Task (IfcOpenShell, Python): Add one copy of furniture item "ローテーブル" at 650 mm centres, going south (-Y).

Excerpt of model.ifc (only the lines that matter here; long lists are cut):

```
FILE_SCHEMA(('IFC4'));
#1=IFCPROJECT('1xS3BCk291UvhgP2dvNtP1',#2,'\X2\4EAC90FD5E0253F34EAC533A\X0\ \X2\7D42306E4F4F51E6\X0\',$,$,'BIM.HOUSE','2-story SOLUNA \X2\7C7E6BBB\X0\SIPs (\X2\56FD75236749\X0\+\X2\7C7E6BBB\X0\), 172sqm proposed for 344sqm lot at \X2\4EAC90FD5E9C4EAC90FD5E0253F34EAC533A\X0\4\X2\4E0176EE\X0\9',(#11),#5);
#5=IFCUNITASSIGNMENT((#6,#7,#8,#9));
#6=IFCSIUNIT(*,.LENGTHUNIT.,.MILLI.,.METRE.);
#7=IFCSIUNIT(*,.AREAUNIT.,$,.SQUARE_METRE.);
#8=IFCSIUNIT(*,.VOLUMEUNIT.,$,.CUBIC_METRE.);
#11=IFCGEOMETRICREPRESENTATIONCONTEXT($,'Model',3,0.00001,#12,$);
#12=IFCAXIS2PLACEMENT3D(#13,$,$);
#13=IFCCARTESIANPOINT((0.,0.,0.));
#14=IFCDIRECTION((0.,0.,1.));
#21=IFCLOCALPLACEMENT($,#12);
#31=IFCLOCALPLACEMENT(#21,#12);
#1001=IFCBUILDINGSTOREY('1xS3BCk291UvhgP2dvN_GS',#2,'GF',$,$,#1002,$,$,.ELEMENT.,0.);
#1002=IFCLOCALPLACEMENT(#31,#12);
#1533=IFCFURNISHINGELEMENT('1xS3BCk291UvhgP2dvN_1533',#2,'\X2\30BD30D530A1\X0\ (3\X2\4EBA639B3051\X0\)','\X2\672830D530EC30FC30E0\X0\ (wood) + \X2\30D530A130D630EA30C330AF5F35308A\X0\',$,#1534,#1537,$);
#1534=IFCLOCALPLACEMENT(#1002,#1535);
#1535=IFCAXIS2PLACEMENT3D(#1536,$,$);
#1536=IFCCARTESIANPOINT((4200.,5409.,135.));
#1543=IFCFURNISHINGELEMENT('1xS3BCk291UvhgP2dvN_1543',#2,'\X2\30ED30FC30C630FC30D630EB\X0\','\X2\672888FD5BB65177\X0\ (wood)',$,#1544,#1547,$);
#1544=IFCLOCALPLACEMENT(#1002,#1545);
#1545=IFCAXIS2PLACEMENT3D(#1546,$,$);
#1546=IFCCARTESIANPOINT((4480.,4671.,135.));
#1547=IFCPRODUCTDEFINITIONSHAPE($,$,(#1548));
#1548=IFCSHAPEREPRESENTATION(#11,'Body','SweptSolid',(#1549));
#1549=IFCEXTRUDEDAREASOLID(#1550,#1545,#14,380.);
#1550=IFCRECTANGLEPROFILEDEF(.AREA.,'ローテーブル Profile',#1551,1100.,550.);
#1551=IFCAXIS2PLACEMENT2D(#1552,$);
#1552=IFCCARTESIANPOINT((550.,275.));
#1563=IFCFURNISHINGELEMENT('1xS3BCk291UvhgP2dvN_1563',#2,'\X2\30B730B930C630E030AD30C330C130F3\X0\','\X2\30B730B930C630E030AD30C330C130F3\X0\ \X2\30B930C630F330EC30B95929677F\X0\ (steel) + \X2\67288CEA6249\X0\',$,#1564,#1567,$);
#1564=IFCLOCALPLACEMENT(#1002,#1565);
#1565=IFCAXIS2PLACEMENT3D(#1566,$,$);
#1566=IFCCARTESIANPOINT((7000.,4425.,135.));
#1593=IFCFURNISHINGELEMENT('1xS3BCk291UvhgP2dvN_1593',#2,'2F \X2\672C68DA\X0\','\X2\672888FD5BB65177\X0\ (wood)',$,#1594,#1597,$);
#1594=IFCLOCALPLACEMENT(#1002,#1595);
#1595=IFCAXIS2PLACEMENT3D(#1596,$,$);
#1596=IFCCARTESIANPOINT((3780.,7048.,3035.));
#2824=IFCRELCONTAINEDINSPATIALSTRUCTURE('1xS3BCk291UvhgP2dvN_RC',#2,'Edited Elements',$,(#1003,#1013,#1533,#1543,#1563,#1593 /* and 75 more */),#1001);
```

```python
import numpy as np
import ifcopenshell
import ifcopenshell.api.geometry
import ifcopenshell.api.root
import ifcopenshell.util.element
import ifcopenshell.util.placement
import ifcopenshell.util.unit

model = ifcopenshell.open("model.ifc")
unit_scale = ifcopenshell.util.unit.calculate_unit_scale(model)


def reuse_history(source, copy):
    """copy_class also copies each property set's owner history, people and application; keep the originals."""
    for rel in copy.IsDefinedBy:
        if rel.is_a("IfcRelDefinesByProperties") and (history := rel.RelatingPropertyDefinition.OwnerHistory):
            rel.RelatingPropertyDefinition.OwnerHistory = source.OwnerHistory
            ifcopenshell.util.element.remove_deep2(model, history)


source = model.by_id(1543)
base = ifcopenshell.util.placement.get_local_placement(source.ObjectPlacement)
step = np.array([0.0, -1.0, 0.0]) * 0.65 / unit_scale

for i in range(1, 2):
    copy = ifcopenshell.api.root.copy_class(model, product=source)
    copy.Representation = ifcopenshell.util.element.copy_deep(
        model, source.Representation, exclude=["IfcGeometricRepresentationContext", "IfcRepresentationMap"]
    )
    reuse_history(source, copy)
    matrix = base.copy()
    matrix[:3, 3] += i * step
    print("added at", matrix[:3, 3].round(3) + 0.0)
    ifcopenshell.api.geometry.edit_object_placement(model, product=copy, matrix=matrix, is_si=False)

model.write("model-out.ifc")
```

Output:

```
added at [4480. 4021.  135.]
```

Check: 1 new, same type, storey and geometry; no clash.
